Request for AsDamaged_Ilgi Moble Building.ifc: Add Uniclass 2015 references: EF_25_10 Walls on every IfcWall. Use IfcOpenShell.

First a look at what the model holds.

```python
import ifcopenshell

model = ifcopenshell.open("AsDamaged_Ilgi Moble Building.ifc")
print(model.schema)
print("classifications:", [c.Name for c in model.by_type("IfcClassification")])
for ifc_class in ("IfcDoor", "IfcRoof", "IfcStair", "IfcWall", "IfcWindow"):
    print(ifc_class, len(model.by_type(ifc_class)))
```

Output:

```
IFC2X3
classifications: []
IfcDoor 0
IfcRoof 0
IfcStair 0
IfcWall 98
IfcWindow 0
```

```python
import ifcopenshell
import ifcopenshell.api.classification

model = ifcopenshell.open("AsDamaged_Ilgi Moble Building.ifc")

# IFC2X3 requires Source and Edition and has no link from the project to the system.
system = model.create_entity("IfcClassification", Source="NBS", Edition="2015", Name="Uniclass 2015")

codes = {
    "IfcWall": ("EF_25_10", "Walls"),
}
for ifc_class, (code, name) in codes.items():
    products = model.by_type(ifc_class)
    ifcopenshell.api.classification.add_reference(
        model, products=products, classification=system, identification=code, name=name
    )
    print(code, len(products))

model.write("AsDamaged_Ilgi Moble Building_rev.ifc")
```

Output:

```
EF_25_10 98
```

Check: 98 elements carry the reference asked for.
